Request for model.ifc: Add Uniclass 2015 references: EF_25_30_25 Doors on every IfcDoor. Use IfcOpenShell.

First a look at what the model holds.

```python
import ifcopenshell

model = ifcopenshell.open("model.ifc")
print(model.schema)
print("classifications:", [c.Name for c in model.by_type("IfcClassification")])
for ifc_class in ("IfcDoor", "IfcRoof", "IfcStair", "IfcWall", "IfcWindow"):
    print(ifc_class, len(model.by_type(ifc_class)))
```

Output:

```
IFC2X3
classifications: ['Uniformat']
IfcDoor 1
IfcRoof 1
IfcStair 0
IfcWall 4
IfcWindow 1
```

```python
import ifcopenshell
import ifcopenshell.api.classification

model = ifcopenshell.open("model.ifc")

# IFC2X3 requires Source and Edition and has no link from the project to the system.
system = model.create_entity("IfcClassification", Source="NBS", Edition="2015", Name="Uniclass 2015")

codes = {
    "IfcDoor": ("EF_25_30_25", "Doors"),
}
for ifc_class, (code, name) in codes.items():
    products = model.by_type(ifc_class)
    ifcopenshell.api.classification.add_reference(
        model, products=products, classification=system, identification=code, name=name
    )
    print(code, len(products))

model.write("model_updated.ifc")
```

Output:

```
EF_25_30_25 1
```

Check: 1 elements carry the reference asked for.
